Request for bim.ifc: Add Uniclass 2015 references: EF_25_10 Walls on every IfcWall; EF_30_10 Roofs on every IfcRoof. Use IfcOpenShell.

First a look at what the model holds.

```python
import ifcopenshell

model = ifcopenshell.open("bim.ifc")
print(model.schema)
print("classifications:", [c.Name for c in model.by_type("IfcClassification")])
for ifc_class in ("IfcDoor", "IfcRoof", "IfcStair", "IfcWall", "IfcWindow"):
    print(ifc_class, len(model.by_type(ifc_class)))
```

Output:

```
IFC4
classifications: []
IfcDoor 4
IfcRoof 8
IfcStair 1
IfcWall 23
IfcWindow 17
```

```python
import ifcopenshell
import ifcopenshell.api.classification

model = ifcopenshell.open("bim.ifc")

system = ifcopenshell.api.classification.add_classification(model, classification="Uniclass 2015")

codes = {
    "IfcWall": ("EF_25_10", "Walls"),
    "IfcRoof": ("EF_30_10", "Roofs"),
}
for ifc_class, (code, name) in codes.items():
    products = model.by_type(ifc_class)
    ifcopenshell.api.classification.add_reference(
        model, products=products, classification=system, identification=code, name=name
    )
    print(code, len(products))

model.write("bim_rev.ifc")
```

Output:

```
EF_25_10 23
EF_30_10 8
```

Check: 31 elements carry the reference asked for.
